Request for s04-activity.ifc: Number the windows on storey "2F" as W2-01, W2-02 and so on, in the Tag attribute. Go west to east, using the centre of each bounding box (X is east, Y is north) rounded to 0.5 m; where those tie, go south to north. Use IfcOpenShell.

First a look at what the model holds.

```python
import ifcopenshell
import ifcopenshell.util.element
import ifcopenshell.util.placement

model = ifcopenshell.open("s04-activity.ifc")
print(model.schema)
storey = next(s for s in model.by_type("IfcBuildingStorey") if s.Name == "2F")
windows = [e for e in ifcopenshell.util.element.get_decomposition(storey) if e.is_a("IfcWindow")]
for e in sorted(windows, key=lambda e: e.id()):
    origin = ifcopenshell.util.placement.get_local_placement(e.ObjectPlacement)[:3, 3]
    print(e.id(), e.Tag, e.Name, origin.round(2) + 0.0, sep=" | ")
```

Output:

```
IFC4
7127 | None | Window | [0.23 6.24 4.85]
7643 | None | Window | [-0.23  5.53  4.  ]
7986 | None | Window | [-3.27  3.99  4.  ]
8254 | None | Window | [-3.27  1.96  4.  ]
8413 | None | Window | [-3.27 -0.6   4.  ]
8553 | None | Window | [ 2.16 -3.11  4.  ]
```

```python
import ifcopenshell
import ifcopenshell.geom
import ifcopenshell.util.element
import ifcopenshell.util.shape

model = ifcopenshell.open("s04-activity.ifc")
settings = ifcopenshell.geom.settings()
settings.set("use-world-coords", True)


def centre(element):
    shape = ifcopenshell.geom.create_shape(settings, element)
    return ifcopenshell.util.shape.get_bbox_centroid(shape.geometry)


storey = next(s for s in model.by_type("IfcBuildingStorey") if s.Name == "2F")
windows = [e for e in ifcopenshell.util.element.get_decomposition(storey) if e.is_a("IfcWindow")]

# Insertion points can sit at a corner or the storey origin, so sort by the geometry (in metres).
centres = {e: centre(e) for e in windows}
windows.sort(key=lambda e: (round(centres[e][0] / 0.5), centres[e][1]))

for i, e in enumerate(windows, start=1):
    number = f"W2-{i:02d}"
    e.Tag = number
    print(e.id(), number)

model.write("s04-activity-out.ifc")
```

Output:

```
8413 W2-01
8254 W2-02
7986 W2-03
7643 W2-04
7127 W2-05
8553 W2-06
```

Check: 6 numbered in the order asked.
